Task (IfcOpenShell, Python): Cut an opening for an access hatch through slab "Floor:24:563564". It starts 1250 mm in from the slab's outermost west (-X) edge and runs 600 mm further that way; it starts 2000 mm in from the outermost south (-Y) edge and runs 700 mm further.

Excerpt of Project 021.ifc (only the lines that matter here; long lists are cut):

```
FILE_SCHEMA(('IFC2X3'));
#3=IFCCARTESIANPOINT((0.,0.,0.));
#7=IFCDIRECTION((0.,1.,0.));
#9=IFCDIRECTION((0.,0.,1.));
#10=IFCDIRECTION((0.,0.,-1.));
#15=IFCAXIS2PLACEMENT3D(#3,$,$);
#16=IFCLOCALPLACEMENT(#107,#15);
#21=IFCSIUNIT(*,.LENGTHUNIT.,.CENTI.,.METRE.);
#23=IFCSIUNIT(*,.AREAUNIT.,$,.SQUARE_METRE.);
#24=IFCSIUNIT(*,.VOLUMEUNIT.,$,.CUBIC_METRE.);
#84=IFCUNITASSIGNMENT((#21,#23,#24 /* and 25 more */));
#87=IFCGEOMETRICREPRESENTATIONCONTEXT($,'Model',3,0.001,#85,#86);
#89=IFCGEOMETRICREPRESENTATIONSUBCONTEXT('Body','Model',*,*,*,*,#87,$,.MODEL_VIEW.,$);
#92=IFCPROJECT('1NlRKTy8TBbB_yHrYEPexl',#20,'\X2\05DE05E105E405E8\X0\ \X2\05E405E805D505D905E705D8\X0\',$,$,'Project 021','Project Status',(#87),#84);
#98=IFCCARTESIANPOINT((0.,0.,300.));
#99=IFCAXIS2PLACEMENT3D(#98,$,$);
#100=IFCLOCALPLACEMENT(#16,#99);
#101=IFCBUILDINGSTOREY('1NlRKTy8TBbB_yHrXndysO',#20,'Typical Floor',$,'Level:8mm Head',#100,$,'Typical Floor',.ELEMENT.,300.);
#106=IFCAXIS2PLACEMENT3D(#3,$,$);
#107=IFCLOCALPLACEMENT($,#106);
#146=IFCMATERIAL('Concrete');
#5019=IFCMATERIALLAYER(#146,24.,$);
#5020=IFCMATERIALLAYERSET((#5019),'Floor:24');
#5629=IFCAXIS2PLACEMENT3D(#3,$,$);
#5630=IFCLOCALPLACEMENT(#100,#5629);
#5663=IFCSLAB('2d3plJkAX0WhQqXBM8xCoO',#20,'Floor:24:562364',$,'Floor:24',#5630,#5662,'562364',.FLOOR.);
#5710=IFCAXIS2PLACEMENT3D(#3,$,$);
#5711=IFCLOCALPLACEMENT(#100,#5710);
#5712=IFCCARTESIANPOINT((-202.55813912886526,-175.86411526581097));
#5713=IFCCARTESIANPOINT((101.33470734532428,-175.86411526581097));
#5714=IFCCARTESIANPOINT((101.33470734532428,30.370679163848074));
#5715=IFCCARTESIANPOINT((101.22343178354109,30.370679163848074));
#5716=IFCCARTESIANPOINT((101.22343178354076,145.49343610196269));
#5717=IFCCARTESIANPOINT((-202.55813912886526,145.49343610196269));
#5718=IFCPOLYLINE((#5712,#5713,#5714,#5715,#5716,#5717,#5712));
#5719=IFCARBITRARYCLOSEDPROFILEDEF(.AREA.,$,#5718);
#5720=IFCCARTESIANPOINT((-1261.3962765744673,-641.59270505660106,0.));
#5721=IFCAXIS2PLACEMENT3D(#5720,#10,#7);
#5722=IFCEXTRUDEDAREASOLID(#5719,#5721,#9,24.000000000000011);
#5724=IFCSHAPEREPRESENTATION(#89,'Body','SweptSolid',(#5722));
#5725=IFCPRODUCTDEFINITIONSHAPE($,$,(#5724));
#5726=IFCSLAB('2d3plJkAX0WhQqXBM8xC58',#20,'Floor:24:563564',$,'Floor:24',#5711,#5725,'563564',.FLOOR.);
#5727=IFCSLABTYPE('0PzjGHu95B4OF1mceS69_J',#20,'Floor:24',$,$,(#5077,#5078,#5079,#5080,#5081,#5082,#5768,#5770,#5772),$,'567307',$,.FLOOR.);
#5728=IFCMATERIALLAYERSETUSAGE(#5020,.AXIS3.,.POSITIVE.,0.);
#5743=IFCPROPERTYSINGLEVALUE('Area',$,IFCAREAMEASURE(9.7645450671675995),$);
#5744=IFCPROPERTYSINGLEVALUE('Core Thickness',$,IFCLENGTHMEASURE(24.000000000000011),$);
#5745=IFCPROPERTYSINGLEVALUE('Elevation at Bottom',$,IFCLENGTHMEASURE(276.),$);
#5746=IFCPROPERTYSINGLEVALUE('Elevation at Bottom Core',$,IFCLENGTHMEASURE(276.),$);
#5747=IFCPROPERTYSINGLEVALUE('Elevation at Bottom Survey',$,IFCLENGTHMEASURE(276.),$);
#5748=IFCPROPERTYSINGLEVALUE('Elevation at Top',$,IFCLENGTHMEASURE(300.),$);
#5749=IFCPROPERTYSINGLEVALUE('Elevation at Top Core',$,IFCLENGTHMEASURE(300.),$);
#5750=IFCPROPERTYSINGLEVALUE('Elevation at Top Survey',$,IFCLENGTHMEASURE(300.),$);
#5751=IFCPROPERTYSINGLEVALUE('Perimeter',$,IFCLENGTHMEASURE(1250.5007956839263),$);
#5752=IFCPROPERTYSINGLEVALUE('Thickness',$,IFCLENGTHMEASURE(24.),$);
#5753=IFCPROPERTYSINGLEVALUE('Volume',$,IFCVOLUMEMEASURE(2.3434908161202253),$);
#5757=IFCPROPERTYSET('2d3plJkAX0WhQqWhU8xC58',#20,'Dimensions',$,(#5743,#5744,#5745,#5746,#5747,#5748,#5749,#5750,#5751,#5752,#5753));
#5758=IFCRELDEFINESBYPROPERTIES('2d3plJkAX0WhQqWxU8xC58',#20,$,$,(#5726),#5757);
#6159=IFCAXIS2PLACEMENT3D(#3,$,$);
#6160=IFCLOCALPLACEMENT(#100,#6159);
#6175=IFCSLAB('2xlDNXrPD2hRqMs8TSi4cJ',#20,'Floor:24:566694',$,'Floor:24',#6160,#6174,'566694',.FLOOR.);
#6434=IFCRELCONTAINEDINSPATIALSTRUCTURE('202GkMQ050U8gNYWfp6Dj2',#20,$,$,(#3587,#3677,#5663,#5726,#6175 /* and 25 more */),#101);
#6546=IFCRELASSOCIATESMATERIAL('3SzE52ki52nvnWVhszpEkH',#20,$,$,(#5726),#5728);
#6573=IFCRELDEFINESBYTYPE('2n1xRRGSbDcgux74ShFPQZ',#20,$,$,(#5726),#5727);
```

```python
import numpy as np
import ifcopenshell
import ifcopenshell.api.feature
import ifcopenshell.api.geometry
import ifcopenshell.api.pset
import ifcopenshell.api.root
import ifcopenshell.geom
import ifcopenshell.util.element
import ifcopenshell.util.placement
import ifcopenshell.util.representation
import ifcopenshell.util.shape
import ifcopenshell.util.unit

model = ifcopenshell.open("Project 021.ifc")
unit_scale = ifcopenshell.util.unit.calculate_unit_scale(model)
area_scale = ifcopenshell.util.unit.calculate_unit_scale(model, "AREAUNIT")
volume_scale = ifcopenshell.util.unit.calculate_unit_scale(model, "VOLUMEUNIT")
settings = ifcopenshell.geom.settings()


def volume(element):
    """Net volume in cubic metres, openings subtracted."""
    shape = ifcopenshell.geom.create_shape(settings, element)
    return ifcopenshell.util.shape.get_volume(shape.geometry)


slab = model.by_guid("2d3plJkAX0WhQqXBM8xC58")
before = volume(slab)

# Extent in the slab's own axes, in metres. The edges named are its -X and -Y sides.
slab_shape = ifcopenshell.geom.create_shape(settings, slab)
vertices = ifcopenshell.util.shape.get_vertices(slab_shape.geometry)
x_min, y_min, bottom = vertices.min(axis=0)
top = vertices[:, 2].max()

opening = ifcopenshell.api.root.create_entity(model, ifc_class="IfcOpeningElement", name="Access hatch opening")
context = ifcopenshell.util.representation.get_context(model, "Model", "Body", "MODEL_VIEW")
width, depth = 0.6, 0.7
outline = [(0.0, 0.0), (width, 0.0), (width, depth), (0.0, depth), (0.0, 0.0)]
# Overshoot both faces by 50 mm so the cut is clean.
shape = ifcopenshell.api.geometry.add_slab_representation(
    model, context=context, depth=top - bottom + 0.1, polyline=outline
)
ifcopenshell.api.geometry.assign_representation(model, product=opening, representation=shape)

matrix = ifcopenshell.util.placement.get_local_placement(slab.ObjectPlacement)
matrix[:, 3] = matrix @ np.append(np.array([x_min + 1.25, y_min + 2, bottom - 0.05]) / unit_scale, 1.0)
ifcopenshell.api.geometry.edit_object_placement(model, product=opening, matrix=matrix, is_si=False)
ifcopenshell.api.feature.add_feature(model, feature=opening, element=slab)

after = volume(slab)

# Update the slab's stored quantities.
pset = model.by_id(ifcopenshell.util.element.get_pset(slab, "Dimensions", should_inherit=False)["id"])
ifcopenshell.api.pset.edit_pset(model, pset=pset, properties={
    "Area": model.create_entity("IfcAreaMeasure", after / (top - bottom) / area_scale),
    "Volume": model.create_entity("IfcVolumeMeasure", after / volume_scale),
})

print(f"slab volume {before:.3f} -> {after:.3f} m3")

model.write("Project 021-out.ifc")
```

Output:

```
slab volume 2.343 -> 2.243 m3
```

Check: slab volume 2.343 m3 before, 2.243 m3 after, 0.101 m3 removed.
